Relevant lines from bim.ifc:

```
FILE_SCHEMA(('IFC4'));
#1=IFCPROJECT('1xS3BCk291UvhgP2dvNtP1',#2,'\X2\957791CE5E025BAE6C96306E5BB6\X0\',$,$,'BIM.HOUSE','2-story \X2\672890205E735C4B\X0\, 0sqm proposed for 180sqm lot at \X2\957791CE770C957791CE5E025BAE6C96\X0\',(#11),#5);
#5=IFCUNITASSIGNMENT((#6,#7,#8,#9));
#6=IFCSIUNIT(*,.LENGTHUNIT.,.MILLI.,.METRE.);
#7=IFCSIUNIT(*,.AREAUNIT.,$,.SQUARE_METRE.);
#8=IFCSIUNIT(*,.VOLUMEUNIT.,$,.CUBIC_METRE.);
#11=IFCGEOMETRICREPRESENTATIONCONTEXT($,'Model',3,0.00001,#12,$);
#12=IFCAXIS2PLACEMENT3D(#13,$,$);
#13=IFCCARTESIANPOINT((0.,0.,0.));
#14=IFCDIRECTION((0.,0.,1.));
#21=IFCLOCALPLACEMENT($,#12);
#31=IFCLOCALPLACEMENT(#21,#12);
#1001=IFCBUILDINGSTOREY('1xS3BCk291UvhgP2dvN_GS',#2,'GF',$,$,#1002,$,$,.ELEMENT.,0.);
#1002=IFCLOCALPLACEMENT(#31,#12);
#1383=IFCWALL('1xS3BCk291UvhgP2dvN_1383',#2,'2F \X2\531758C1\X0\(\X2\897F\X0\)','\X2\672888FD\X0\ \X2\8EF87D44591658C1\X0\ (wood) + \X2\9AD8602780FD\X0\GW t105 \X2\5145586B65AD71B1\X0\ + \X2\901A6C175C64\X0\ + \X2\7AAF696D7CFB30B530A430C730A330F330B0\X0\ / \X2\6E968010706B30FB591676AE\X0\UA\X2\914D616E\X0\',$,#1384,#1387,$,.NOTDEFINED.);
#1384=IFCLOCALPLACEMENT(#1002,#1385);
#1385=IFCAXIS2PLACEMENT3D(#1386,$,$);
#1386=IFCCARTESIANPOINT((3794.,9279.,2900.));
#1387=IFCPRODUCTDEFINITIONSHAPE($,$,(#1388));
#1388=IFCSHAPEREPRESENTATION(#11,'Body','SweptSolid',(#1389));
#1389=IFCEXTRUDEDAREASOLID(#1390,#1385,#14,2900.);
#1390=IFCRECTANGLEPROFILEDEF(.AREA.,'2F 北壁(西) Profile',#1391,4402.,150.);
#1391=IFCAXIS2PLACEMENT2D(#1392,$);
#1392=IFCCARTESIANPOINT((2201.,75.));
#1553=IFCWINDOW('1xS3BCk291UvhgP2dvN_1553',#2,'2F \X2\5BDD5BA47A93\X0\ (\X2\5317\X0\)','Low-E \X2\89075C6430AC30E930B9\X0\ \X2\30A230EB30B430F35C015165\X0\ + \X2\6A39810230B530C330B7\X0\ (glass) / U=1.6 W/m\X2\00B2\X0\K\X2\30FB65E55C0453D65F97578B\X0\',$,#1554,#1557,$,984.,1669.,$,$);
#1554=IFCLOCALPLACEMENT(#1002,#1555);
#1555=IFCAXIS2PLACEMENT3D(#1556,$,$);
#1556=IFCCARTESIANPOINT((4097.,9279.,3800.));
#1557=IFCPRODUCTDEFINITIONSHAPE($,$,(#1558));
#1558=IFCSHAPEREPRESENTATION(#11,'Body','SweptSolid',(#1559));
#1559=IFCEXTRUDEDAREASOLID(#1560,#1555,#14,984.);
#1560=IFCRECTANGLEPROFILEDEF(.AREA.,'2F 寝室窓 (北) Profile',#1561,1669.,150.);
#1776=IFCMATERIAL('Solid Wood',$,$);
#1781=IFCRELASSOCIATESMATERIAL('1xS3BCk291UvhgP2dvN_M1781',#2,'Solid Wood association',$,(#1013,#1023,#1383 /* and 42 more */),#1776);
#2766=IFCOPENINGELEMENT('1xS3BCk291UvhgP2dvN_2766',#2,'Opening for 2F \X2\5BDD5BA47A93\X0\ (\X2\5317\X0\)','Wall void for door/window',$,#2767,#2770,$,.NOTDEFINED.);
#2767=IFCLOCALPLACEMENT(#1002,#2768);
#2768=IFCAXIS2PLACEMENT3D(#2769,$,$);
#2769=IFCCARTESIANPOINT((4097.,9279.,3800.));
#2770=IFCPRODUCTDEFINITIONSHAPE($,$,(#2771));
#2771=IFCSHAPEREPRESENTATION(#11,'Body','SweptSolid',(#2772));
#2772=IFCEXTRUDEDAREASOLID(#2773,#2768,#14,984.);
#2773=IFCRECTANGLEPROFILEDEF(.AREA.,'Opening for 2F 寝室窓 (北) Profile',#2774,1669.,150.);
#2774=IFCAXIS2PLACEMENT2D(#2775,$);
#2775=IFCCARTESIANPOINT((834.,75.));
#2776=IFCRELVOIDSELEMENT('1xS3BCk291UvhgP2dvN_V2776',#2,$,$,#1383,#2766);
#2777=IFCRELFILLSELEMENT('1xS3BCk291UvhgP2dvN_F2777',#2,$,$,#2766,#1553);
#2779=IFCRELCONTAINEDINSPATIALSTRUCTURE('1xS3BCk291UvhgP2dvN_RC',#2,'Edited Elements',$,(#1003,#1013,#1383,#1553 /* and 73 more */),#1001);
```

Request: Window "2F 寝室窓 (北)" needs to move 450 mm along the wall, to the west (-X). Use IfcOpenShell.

```python
import ifcopenshell
import ifcopenshell.api.geometry
import ifcopenshell.util.placement

model = ifcopenshell.open("bim.ifc")

window = model.by_guid("1xS3BCk291UvhgP2dvN_1553")
opening = window.FillsVoids[0].RelatingOpeningElement
wall = opening.VoidsElements[0].RelatingBuildingElement

wall_matrix = ifcopenshell.util.placement.get_local_placement(wall.ObjectPlacement)
shift = wall_matrix[:3, 0] * -450.0
before = ifcopenshell.util.placement.get_local_placement(window.ObjectPlacement)[:3, 3].copy()

# The window is not placed relative to its opening, so move both.
for product in (opening, window):
    matrix = ifcopenshell.util.placement.get_local_placement(product.ObjectPlacement)
    matrix[:3, 3] += shift
    ifcopenshell.api.geometry.edit_object_placement(model, product=product, matrix=matrix, is_si=False)

after = ifcopenshell.util.placement.get_local_placement(window.ObjectPlacement)[:3, 3]
print("window moved by", (after - before).round(3) + 0.0)

model.write("bim_v2.ifc")
```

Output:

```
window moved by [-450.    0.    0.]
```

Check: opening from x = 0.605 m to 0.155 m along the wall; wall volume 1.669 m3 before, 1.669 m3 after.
